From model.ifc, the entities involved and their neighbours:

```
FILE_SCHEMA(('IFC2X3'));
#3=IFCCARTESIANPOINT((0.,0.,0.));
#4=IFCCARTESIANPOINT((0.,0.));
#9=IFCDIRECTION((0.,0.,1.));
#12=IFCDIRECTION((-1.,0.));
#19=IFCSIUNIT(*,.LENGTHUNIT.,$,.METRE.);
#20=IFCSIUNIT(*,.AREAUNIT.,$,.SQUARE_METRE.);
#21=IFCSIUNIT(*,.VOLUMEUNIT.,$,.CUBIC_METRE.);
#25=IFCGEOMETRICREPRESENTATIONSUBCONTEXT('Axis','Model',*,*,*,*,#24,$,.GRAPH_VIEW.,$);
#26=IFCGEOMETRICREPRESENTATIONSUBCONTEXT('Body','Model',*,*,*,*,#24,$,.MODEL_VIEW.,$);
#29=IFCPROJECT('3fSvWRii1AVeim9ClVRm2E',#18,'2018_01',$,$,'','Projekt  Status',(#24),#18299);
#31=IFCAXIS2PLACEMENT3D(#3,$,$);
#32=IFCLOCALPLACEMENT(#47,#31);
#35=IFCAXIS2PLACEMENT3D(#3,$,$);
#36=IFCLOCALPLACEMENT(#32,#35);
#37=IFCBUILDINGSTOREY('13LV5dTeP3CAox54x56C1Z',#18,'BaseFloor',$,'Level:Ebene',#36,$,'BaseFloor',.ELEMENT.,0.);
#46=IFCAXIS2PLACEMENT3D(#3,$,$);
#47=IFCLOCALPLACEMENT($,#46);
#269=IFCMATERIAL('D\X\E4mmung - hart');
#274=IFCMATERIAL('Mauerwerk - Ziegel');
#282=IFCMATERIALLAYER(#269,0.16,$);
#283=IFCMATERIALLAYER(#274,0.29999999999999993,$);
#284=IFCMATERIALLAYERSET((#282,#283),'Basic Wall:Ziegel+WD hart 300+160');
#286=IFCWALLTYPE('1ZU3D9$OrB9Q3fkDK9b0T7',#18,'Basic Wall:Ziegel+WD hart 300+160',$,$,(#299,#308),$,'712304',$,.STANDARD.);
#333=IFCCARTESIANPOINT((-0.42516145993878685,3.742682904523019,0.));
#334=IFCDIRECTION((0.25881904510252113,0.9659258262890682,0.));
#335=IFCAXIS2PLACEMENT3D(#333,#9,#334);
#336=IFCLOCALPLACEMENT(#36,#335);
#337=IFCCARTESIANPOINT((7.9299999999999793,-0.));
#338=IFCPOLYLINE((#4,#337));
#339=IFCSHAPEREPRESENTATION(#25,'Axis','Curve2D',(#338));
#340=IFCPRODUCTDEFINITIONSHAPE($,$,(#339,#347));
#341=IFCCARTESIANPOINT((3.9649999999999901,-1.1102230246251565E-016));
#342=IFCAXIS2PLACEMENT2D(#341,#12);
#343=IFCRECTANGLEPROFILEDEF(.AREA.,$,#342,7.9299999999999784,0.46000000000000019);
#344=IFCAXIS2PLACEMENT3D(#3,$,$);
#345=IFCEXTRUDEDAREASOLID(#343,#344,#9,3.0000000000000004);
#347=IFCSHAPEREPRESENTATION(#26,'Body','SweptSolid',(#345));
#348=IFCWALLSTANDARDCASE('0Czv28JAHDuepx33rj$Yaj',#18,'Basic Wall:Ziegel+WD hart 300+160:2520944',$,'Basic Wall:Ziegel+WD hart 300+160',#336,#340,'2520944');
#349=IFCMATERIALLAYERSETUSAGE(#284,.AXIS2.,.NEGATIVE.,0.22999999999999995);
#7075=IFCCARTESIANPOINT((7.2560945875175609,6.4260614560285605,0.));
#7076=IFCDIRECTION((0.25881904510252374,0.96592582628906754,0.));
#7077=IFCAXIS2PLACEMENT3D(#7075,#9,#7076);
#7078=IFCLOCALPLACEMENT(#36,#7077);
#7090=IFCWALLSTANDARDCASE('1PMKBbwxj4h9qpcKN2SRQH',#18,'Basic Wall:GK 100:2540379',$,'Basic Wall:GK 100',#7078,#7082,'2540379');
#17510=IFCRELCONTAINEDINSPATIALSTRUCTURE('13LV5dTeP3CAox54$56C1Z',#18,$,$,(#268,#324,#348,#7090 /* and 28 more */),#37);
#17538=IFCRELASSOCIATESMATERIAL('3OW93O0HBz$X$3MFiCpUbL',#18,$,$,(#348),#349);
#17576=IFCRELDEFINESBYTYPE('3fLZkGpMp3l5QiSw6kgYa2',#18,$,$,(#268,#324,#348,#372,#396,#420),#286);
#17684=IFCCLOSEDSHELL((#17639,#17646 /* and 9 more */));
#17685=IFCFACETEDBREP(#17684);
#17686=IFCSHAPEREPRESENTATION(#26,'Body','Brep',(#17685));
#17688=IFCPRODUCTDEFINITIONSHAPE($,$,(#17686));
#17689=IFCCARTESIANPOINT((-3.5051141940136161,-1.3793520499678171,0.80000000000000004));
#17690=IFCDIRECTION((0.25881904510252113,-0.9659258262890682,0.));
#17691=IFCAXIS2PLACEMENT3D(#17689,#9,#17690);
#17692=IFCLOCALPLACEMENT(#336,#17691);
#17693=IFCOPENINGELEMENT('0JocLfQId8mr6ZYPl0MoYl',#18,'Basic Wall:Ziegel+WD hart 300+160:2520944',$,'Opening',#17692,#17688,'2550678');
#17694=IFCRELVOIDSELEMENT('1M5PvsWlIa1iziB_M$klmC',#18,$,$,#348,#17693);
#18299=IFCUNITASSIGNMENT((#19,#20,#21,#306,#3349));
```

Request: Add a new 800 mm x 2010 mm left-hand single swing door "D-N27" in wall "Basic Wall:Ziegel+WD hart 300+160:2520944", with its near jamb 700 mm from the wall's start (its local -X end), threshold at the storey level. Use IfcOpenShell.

```python
import numpy as np
import ifcopenshell
import ifcopenshell.api.feature
import ifcopenshell.api.geometry
import ifcopenshell.api.root
import ifcopenshell.api.spatial
import ifcopenshell.api.type
import ifcopenshell.geom
import ifcopenshell.util.element
import ifcopenshell.util.placement
import ifcopenshell.util.representation
import ifcopenshell.util.shape
import ifcopenshell.util.unit

model = ifcopenshell.open("model.ifc")
unit_scale = ifcopenshell.util.unit.calculate_unit_scale(model)
settings = ifcopenshell.geom.settings()


def volume(element):
    """Net volume in cubic metres, openings subtracted."""
    shape = ifcopenshell.geom.create_shape(settings, element)
    return ifcopenshell.util.shape.get_volume(shape.geometry)


wall = model.by_guid("0Czv28JAHDuepx33rj$Yaj")
storey = ifcopenshell.util.element.get_container(wall, ifc_class="IfcBuildingStorey")
context = ifcopenshell.util.representation.get_context(model, "Model", "Body", "MODEL_VIEW")
before = volume(wall)

width, height, from_end, sill = 0.8, 2.01, 0.7, 0.0  # metres

# The wall runs along its own X axis, and the end named is its -X end.
wall_shape = ifcopenshell.geom.create_shape(settings, wall)
x, y, z = ifcopenshell.util.shape.get_vertices(wall_shape.geometry).T
start = x.min() + from_end
face, thickness = float(y.min()), float(y.max() - y.min())
wall_matrix = ifcopenshell.util.placement.get_local_placement(wall.ObjectPlacement)
level = ifcopenshell.util.placement.get_local_placement(storey.ObjectPlacement)[2, 3]


def in_wall(x, y):
    """Placement at x, y metres in the wall's axes, at sill height."""
    matrix = wall_matrix.copy()
    matrix[:, 3] = wall_matrix @ np.array([x / unit_scale, y / unit_scale, 0.0, 1.0])
    matrix[2, 3] = level + sill / unit_scale
    return matrix


# Opening: a box that overshoots both wall faces by 50 mm.
opening = ifcopenshell.api.root.create_entity(model, ifc_class="IfcOpeningElement")
box = ifcopenshell.api.geometry.add_wall_representation(
    model, context=context, length=width, height=height, thickness=thickness + 0.1
)
ifcopenshell.api.geometry.assign_representation(model, product=opening, representation=box)
ifcopenshell.api.geometry.edit_object_placement(model, product=opening, matrix=in_wall(start, face - 0.05), is_si=False)
ifcopenshell.api.feature.add_feature(model, feature=opening, element=wall)

door = ifcopenshell.api.root.create_entity(model, ifc_class="IfcDoor", name="D-N27")
door.OverallWidth, door.OverallHeight = width / unit_scale, height / unit_scale
body = ifcopenshell.api.geometry.add_door_representation(
    model,
    context=context,
    overall_width=door.OverallWidth,
    overall_height=door.OverallHeight,
    operation_type="SINGLE_SWING_LEFT",
    lining_properties={"LiningDepth": thickness / unit_scale, "ThresholdDepth": thickness / unit_scale},
)
ifcopenshell.api.geometry.assign_representation(model, product=door, representation=body)
ifcopenshell.api.spatial.assign_container(model, products=[door], relating_structure=storey)
fills = ifcopenshell.api.feature.add_filling(model, opening=opening, element=door)
fills.OwnerHistory = door.OwnerHistory  # required in IFC2X3

# IFC2X3 keeps the operation on the door style.
style = ifcopenshell.api.root.create_entity(model, ifc_class="IfcDoorStyle", name="D-N27")
style.OperationType, style.ConstructionType = "SINGLE_SWING_LEFT", "NOTDEFINED"
style.ParameterTakesPrecedence = style.Sizeable = False
ifcopenshell.api.type.assign_type(model, related_objects=[door], relating_type=style)

# The lining spans the wall, so the door starts at the wall face.
ifcopenshell.api.geometry.edit_object_placement(model, product=door, matrix=in_wall(start, face), is_si=False)

after = volume(wall)

print(f"wall volume {before:.3f} -> {after:.3f} m3")

model.write("model-out.ifc")
```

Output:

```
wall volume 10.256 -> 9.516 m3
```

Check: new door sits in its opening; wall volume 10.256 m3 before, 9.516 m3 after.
